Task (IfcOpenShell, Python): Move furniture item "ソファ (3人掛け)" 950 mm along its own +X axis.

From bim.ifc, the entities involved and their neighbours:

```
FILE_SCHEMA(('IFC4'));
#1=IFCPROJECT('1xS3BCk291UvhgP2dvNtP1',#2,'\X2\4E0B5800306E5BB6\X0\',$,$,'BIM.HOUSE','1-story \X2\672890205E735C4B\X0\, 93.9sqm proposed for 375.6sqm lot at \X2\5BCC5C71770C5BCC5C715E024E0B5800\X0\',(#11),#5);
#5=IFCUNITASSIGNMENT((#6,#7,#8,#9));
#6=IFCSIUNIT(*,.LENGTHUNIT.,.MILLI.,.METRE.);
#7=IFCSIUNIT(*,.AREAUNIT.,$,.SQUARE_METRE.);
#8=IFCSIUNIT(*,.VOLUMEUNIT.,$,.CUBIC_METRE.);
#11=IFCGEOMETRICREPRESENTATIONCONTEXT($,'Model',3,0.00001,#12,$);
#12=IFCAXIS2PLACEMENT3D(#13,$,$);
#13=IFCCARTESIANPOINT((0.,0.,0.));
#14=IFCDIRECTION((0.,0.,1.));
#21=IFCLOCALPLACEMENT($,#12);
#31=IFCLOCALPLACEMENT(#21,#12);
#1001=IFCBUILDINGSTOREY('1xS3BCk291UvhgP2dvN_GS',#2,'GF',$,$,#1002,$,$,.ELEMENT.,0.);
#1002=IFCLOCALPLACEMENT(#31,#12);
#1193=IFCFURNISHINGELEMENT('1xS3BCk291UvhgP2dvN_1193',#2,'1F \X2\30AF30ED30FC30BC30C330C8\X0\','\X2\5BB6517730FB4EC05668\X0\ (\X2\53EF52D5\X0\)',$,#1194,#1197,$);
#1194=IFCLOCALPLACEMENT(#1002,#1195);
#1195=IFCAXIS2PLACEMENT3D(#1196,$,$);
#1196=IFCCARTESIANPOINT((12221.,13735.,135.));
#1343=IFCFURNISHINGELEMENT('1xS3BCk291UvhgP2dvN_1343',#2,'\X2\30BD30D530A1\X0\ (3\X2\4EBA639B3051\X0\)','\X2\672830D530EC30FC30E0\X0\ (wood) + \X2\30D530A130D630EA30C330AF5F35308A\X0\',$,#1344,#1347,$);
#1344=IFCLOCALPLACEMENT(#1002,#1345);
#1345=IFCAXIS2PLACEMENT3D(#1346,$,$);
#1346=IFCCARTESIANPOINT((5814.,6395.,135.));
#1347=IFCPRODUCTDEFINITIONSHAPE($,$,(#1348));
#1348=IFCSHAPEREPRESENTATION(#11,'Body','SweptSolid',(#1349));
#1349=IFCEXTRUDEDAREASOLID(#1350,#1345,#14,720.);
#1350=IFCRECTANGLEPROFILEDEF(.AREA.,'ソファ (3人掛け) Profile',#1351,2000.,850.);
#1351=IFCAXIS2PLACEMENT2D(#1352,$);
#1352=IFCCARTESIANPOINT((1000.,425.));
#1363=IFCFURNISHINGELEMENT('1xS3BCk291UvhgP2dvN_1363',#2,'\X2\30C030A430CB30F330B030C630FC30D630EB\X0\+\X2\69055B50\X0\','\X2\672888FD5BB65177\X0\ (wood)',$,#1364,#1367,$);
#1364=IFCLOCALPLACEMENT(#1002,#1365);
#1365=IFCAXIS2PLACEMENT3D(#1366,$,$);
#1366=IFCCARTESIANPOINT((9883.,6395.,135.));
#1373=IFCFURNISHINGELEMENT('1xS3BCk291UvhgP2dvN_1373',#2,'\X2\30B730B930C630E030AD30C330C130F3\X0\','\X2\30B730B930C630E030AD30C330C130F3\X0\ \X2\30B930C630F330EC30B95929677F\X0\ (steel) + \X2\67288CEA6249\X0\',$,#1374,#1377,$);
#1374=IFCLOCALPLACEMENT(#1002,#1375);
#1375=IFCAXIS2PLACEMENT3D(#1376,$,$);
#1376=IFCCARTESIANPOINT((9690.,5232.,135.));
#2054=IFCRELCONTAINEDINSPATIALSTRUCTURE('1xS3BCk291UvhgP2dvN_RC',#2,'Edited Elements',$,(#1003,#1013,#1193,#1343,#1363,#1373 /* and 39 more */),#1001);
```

```python
import ifcopenshell
import ifcopenshell.api.geometry
import ifcopenshell.util.placement
import ifcopenshell.util.unit

model = ifcopenshell.open("bim.ifc")
unit_scale = ifcopenshell.util.unit.calculate_unit_scale(model)

item = model.by_guid("1xS3BCk291UvhgP2dvN_1343")
matrix = ifcopenshell.util.placement.get_local_placement(item.ObjectPlacement)
matrix[:3, 3] += matrix[:3, 0] * 0.95 / unit_scale
ifcopenshell.api.geometry.edit_object_placement(model, product=item, matrix=matrix, is_si=False)

print(ifcopenshell.util.placement.get_local_placement(item.ObjectPlacement).round(3) + 0.0)

model.write("bim-out.ifc")
```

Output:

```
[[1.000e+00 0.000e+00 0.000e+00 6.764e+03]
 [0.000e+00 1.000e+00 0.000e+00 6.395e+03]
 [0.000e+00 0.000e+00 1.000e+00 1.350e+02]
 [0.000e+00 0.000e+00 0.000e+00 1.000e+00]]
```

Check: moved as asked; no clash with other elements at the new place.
